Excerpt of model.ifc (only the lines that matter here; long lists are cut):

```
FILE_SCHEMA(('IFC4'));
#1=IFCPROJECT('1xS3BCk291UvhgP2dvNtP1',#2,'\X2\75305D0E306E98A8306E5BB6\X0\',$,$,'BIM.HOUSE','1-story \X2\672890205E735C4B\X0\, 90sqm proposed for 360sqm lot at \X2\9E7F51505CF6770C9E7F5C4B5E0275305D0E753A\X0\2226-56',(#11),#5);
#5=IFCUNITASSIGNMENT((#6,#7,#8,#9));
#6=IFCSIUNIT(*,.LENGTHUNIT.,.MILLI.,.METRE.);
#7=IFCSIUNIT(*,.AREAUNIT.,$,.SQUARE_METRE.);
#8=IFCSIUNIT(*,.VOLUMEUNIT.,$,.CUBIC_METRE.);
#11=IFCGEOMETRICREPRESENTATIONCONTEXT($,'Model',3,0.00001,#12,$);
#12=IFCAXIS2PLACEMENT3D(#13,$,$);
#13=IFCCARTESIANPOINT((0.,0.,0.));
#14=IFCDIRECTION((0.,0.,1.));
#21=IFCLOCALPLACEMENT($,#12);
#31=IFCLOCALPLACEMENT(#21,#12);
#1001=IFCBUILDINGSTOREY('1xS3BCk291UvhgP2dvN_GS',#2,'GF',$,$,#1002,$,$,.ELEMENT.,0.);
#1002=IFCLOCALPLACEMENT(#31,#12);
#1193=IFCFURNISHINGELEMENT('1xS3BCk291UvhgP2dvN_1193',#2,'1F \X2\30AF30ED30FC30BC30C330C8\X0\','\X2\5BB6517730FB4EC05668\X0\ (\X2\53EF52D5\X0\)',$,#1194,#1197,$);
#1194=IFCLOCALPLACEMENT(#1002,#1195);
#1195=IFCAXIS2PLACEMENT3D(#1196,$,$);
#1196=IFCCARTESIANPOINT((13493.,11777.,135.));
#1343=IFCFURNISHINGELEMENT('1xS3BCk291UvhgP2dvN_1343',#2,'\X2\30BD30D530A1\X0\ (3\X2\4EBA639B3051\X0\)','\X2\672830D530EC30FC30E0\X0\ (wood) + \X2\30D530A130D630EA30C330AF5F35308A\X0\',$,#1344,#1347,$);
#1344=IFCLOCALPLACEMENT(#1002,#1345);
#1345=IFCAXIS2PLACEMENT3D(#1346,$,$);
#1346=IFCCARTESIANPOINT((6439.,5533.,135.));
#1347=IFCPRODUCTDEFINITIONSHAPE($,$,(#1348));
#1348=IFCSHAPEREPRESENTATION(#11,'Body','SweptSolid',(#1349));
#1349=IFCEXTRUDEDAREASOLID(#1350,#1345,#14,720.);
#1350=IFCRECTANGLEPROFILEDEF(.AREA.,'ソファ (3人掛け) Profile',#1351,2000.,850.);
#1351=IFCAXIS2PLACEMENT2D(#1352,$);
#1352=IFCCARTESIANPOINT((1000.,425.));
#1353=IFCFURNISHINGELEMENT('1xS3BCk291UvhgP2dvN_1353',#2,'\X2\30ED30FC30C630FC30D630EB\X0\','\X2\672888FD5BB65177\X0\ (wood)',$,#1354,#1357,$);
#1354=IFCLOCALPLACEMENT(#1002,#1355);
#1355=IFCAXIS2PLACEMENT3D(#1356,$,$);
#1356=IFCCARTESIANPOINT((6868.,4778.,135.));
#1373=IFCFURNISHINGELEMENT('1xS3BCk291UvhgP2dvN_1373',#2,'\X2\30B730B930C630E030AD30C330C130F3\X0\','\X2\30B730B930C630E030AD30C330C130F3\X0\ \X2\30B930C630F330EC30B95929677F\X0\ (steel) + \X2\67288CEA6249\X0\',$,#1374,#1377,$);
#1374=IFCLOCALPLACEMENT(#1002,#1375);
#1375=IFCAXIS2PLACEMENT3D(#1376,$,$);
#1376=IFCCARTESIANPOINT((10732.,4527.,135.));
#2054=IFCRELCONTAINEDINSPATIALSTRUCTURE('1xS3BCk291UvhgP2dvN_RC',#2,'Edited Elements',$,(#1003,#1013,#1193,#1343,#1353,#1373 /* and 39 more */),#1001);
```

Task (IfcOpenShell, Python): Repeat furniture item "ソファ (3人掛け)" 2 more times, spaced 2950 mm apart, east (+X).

```python
import numpy as np
import ifcopenshell
import ifcopenshell.api.geometry
import ifcopenshell.api.root
import ifcopenshell.util.element
import ifcopenshell.util.placement
import ifcopenshell.util.unit

model = ifcopenshell.open("model.ifc")
unit_scale = ifcopenshell.util.unit.calculate_unit_scale(model)


def reuse_history(source, copy):
    """copy_class also copies each property set's owner history, people and application; keep the originals."""
    for rel in copy.IsDefinedBy:
        if rel.is_a("IfcRelDefinesByProperties") and (history := rel.RelatingPropertyDefinition.OwnerHistory):
            rel.RelatingPropertyDefinition.OwnerHistory = source.OwnerHistory
            ifcopenshell.util.element.remove_deep2(model, history)


source = model.by_guid("1xS3BCk291UvhgP2dvN_1343")
base = ifcopenshell.util.placement.get_local_placement(source.ObjectPlacement)
step = np.array([1.0, 0.0, 0.0]) * 2.95 / unit_scale

for i in range(1, 3):
    copy = ifcopenshell.api.root.copy_class(model, product=source)
    copy.Representation = ifcopenshell.util.element.copy_deep(
        model, source.Representation, exclude=["IfcGeometricRepresentationContext", "IfcRepresentationMap"]
    )
    reuse_history(source, copy)
    matrix = base.copy()
    matrix[:3, 3] += i * step
    print("added at", matrix[:3, 3].round(3) + 0.0)
    ifcopenshell.api.geometry.edit_object_placement(model, product=copy, matrix=matrix, is_si=False)

model.write("model_updated.ifc")
```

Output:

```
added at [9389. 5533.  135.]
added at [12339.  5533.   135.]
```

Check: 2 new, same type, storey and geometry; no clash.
